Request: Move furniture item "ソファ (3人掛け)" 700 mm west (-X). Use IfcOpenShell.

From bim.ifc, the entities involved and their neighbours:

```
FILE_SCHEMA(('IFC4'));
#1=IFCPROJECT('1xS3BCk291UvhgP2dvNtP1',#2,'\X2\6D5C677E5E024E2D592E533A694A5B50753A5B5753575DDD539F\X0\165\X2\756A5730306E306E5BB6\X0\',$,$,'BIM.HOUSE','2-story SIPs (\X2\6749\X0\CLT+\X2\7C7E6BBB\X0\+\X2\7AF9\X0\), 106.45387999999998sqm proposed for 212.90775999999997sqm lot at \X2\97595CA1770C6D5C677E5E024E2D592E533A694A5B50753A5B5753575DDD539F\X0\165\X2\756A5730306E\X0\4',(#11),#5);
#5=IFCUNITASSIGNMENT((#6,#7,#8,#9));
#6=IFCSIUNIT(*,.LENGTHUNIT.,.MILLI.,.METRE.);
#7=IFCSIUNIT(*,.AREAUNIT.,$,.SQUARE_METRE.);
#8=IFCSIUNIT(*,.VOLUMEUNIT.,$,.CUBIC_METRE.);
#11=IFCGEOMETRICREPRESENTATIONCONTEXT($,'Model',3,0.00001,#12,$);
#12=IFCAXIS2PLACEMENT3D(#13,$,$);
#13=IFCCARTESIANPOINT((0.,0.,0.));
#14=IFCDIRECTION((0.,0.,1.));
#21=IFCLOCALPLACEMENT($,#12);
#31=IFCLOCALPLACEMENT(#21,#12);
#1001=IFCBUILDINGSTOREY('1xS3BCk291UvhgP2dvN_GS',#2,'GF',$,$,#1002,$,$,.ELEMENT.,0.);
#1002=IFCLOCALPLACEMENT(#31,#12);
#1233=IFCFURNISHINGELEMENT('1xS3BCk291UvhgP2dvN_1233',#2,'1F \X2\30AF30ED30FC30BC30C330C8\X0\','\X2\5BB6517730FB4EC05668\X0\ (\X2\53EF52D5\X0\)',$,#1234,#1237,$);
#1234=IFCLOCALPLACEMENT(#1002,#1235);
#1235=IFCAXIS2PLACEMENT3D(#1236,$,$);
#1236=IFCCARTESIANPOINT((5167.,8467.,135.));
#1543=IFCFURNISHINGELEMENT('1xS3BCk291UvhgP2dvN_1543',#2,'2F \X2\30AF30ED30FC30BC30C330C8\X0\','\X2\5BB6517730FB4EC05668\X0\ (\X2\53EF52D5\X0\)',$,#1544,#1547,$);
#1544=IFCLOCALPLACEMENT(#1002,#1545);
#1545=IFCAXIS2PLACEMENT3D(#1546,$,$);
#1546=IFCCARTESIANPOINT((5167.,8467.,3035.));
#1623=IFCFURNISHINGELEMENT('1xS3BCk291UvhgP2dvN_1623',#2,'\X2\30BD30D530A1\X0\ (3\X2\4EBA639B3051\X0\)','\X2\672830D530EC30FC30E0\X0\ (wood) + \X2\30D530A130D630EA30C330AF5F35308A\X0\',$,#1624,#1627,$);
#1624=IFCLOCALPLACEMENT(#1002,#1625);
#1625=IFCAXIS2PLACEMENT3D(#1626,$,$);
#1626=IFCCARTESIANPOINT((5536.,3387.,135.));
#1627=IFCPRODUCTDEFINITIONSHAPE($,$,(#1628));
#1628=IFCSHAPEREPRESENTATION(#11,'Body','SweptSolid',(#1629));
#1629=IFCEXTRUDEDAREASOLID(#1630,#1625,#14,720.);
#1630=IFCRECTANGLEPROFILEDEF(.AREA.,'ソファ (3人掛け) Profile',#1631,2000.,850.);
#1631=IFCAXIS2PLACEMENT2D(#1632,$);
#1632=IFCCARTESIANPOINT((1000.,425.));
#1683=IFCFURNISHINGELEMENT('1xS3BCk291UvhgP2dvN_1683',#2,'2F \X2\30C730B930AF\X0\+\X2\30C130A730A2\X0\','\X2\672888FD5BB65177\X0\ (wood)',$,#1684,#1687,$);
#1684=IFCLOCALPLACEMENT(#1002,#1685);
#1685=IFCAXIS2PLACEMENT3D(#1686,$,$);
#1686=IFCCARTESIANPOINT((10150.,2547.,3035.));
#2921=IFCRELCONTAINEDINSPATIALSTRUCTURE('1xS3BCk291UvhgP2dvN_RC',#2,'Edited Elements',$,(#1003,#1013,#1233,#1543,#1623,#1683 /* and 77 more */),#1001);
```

```python
import ifcopenshell
import ifcopenshell.api.geometry
import ifcopenshell.util.placement
import ifcopenshell.util.unit

model = ifcopenshell.open("bim.ifc")
unit_scale = ifcopenshell.util.unit.calculate_unit_scale(model)

item = model.by_id(1623)
matrix = ifcopenshell.util.placement.get_local_placement(item.ObjectPlacement)
matrix[0, 3] -= 0.7 / unit_scale
ifcopenshell.api.geometry.edit_object_placement(model, product=item, matrix=matrix, is_si=False)

print(ifcopenshell.util.placement.get_local_placement(item.ObjectPlacement).round(3) + 0.0)

model.write("bim-out.ifc")
```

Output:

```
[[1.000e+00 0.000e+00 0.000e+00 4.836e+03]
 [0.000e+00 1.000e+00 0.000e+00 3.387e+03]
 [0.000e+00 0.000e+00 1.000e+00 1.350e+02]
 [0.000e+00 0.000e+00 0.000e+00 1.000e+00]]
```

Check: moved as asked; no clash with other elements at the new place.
